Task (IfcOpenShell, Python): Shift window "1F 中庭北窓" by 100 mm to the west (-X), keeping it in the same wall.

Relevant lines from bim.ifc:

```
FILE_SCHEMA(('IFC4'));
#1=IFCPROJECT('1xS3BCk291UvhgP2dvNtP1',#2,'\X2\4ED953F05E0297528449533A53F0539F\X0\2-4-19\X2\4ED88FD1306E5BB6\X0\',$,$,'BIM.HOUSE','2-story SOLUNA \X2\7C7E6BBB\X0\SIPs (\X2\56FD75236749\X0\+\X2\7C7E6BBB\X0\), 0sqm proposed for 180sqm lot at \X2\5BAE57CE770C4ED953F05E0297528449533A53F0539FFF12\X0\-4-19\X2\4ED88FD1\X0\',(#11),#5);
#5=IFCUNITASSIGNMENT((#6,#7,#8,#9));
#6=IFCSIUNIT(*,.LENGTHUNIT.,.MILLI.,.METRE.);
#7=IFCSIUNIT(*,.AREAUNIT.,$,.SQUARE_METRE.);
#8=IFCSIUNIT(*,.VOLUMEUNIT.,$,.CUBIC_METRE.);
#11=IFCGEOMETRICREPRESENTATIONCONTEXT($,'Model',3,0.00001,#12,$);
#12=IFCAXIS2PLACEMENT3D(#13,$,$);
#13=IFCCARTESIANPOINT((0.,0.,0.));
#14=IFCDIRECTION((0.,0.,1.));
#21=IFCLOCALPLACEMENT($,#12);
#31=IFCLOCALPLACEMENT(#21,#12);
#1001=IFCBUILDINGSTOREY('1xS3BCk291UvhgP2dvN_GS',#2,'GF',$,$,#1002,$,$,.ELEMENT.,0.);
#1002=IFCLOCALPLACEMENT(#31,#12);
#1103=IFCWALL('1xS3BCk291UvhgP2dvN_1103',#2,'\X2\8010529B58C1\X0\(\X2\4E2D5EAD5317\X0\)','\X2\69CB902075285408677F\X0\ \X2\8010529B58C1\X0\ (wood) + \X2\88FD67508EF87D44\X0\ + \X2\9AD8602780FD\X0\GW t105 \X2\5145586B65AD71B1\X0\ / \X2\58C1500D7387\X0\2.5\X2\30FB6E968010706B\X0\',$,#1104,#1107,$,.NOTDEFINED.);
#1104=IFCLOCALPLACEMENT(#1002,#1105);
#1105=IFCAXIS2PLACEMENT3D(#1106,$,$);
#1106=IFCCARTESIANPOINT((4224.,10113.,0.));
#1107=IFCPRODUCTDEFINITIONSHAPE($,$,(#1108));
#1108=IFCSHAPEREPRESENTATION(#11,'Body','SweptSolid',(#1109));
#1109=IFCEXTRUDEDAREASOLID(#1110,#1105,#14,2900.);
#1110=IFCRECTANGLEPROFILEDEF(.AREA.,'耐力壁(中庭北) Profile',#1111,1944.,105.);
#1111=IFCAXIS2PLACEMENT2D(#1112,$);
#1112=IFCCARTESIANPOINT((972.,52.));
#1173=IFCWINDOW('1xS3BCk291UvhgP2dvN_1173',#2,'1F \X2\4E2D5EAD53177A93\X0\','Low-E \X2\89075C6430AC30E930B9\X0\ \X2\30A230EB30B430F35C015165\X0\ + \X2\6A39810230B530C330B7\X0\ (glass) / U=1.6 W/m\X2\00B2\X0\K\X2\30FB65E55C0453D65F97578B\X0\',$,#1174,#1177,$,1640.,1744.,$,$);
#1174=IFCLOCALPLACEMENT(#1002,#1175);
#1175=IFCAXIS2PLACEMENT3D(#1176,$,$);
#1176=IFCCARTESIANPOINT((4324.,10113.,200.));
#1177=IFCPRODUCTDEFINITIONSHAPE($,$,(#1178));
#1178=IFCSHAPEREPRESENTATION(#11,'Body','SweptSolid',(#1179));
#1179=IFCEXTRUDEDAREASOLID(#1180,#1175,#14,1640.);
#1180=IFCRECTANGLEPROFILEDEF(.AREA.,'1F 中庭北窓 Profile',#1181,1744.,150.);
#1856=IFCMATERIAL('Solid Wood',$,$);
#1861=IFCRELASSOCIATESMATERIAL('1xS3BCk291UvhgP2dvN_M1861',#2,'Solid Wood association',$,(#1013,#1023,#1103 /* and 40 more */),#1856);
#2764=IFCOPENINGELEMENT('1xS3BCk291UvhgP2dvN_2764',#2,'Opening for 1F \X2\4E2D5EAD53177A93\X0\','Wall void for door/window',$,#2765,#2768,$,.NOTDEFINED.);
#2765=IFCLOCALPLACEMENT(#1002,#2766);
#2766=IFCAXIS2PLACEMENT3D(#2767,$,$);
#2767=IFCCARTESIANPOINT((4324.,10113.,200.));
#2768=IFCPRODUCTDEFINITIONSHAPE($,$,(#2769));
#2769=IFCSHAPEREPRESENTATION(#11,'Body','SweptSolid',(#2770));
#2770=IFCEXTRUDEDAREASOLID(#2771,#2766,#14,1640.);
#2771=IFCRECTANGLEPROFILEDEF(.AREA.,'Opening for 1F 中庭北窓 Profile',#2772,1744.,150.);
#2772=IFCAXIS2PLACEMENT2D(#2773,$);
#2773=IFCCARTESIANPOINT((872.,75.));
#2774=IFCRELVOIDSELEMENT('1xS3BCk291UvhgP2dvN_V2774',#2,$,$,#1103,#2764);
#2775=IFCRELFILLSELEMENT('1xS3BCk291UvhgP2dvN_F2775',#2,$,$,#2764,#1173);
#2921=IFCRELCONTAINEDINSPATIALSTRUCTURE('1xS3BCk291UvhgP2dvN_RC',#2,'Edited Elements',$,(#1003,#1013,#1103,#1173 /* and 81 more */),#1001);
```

```python
import ifcopenshell
import ifcopenshell.api.geometry
import ifcopenshell.util.placement
import ifcopenshell.util.unit

model = ifcopenshell.open("bim.ifc")
unit_scale = ifcopenshell.util.unit.calculate_unit_scale(model)

window = model.by_id(1173)
opening = window.FillsVoids[0].RelatingOpeningElement
wall = opening.VoidsElements[0].RelatingBuildingElement

wall_matrix = ifcopenshell.util.placement.get_local_placement(wall.ObjectPlacement)
shift = wall_matrix[:3, 0] * -0.1 / unit_scale
before = ifcopenshell.util.placement.get_local_placement(window.ObjectPlacement)[:3, 3].copy()

# The window is not placed relative to its opening, so move both.
for product in (opening, window):
    matrix = ifcopenshell.util.placement.get_local_placement(product.ObjectPlacement)
    matrix[:3, 3] += shift
    ifcopenshell.api.geometry.edit_object_placement(model, product=product, matrix=matrix, is_si=False)

after = ifcopenshell.util.placement.get_local_placement(window.ObjectPlacement)[:3, 3]
print("window moved by", (after - before).round(3) + 0.0)

model.write("bim_rev.ifc")
```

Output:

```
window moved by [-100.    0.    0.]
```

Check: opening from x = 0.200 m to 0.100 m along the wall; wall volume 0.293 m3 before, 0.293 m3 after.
